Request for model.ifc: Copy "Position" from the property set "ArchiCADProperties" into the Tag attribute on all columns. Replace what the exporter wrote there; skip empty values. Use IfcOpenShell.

First a look at what the model holds.

```python
import ifcopenshell
import ifcopenshell.util.element

model = ifcopenshell.open("model.ifc")
print(model.schema)
columns = model.by_type("IfcColumn")
print(len(columns), "columns")
for e in columns[:8]:
    source = ifcopenshell.util.element.get_pset(e, "ArchiCADProperties", "Position")
    target = e.Tag
    print(e.id(), repr(source), repr(target), sep=" | ")
```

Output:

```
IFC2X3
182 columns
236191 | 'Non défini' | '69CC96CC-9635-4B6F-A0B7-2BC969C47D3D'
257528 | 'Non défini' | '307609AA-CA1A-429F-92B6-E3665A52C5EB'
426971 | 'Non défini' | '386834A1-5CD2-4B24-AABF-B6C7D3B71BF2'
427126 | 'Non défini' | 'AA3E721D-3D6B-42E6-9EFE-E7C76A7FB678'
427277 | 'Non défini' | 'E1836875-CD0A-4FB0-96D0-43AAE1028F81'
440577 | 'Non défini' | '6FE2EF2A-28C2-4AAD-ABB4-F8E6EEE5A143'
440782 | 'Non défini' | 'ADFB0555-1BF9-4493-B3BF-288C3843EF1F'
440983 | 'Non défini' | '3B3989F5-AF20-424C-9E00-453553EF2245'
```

```python
import ifcopenshell
import ifcopenshell.util.element

model = ifcopenshell.open("model.ifc")

count = 0
for e in model.by_type("IfcColumn"):
    value = ifcopenshell.util.element.get_pset(e, "ArchiCADProperties", "Position")
    current = e.Tag
    if not value or not value.strip() or current == value:
        continue
    e.Tag = value
    count += 1

print(count, "columns updated")

model.write("model_v2.ifc")
```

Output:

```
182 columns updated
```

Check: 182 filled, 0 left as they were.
